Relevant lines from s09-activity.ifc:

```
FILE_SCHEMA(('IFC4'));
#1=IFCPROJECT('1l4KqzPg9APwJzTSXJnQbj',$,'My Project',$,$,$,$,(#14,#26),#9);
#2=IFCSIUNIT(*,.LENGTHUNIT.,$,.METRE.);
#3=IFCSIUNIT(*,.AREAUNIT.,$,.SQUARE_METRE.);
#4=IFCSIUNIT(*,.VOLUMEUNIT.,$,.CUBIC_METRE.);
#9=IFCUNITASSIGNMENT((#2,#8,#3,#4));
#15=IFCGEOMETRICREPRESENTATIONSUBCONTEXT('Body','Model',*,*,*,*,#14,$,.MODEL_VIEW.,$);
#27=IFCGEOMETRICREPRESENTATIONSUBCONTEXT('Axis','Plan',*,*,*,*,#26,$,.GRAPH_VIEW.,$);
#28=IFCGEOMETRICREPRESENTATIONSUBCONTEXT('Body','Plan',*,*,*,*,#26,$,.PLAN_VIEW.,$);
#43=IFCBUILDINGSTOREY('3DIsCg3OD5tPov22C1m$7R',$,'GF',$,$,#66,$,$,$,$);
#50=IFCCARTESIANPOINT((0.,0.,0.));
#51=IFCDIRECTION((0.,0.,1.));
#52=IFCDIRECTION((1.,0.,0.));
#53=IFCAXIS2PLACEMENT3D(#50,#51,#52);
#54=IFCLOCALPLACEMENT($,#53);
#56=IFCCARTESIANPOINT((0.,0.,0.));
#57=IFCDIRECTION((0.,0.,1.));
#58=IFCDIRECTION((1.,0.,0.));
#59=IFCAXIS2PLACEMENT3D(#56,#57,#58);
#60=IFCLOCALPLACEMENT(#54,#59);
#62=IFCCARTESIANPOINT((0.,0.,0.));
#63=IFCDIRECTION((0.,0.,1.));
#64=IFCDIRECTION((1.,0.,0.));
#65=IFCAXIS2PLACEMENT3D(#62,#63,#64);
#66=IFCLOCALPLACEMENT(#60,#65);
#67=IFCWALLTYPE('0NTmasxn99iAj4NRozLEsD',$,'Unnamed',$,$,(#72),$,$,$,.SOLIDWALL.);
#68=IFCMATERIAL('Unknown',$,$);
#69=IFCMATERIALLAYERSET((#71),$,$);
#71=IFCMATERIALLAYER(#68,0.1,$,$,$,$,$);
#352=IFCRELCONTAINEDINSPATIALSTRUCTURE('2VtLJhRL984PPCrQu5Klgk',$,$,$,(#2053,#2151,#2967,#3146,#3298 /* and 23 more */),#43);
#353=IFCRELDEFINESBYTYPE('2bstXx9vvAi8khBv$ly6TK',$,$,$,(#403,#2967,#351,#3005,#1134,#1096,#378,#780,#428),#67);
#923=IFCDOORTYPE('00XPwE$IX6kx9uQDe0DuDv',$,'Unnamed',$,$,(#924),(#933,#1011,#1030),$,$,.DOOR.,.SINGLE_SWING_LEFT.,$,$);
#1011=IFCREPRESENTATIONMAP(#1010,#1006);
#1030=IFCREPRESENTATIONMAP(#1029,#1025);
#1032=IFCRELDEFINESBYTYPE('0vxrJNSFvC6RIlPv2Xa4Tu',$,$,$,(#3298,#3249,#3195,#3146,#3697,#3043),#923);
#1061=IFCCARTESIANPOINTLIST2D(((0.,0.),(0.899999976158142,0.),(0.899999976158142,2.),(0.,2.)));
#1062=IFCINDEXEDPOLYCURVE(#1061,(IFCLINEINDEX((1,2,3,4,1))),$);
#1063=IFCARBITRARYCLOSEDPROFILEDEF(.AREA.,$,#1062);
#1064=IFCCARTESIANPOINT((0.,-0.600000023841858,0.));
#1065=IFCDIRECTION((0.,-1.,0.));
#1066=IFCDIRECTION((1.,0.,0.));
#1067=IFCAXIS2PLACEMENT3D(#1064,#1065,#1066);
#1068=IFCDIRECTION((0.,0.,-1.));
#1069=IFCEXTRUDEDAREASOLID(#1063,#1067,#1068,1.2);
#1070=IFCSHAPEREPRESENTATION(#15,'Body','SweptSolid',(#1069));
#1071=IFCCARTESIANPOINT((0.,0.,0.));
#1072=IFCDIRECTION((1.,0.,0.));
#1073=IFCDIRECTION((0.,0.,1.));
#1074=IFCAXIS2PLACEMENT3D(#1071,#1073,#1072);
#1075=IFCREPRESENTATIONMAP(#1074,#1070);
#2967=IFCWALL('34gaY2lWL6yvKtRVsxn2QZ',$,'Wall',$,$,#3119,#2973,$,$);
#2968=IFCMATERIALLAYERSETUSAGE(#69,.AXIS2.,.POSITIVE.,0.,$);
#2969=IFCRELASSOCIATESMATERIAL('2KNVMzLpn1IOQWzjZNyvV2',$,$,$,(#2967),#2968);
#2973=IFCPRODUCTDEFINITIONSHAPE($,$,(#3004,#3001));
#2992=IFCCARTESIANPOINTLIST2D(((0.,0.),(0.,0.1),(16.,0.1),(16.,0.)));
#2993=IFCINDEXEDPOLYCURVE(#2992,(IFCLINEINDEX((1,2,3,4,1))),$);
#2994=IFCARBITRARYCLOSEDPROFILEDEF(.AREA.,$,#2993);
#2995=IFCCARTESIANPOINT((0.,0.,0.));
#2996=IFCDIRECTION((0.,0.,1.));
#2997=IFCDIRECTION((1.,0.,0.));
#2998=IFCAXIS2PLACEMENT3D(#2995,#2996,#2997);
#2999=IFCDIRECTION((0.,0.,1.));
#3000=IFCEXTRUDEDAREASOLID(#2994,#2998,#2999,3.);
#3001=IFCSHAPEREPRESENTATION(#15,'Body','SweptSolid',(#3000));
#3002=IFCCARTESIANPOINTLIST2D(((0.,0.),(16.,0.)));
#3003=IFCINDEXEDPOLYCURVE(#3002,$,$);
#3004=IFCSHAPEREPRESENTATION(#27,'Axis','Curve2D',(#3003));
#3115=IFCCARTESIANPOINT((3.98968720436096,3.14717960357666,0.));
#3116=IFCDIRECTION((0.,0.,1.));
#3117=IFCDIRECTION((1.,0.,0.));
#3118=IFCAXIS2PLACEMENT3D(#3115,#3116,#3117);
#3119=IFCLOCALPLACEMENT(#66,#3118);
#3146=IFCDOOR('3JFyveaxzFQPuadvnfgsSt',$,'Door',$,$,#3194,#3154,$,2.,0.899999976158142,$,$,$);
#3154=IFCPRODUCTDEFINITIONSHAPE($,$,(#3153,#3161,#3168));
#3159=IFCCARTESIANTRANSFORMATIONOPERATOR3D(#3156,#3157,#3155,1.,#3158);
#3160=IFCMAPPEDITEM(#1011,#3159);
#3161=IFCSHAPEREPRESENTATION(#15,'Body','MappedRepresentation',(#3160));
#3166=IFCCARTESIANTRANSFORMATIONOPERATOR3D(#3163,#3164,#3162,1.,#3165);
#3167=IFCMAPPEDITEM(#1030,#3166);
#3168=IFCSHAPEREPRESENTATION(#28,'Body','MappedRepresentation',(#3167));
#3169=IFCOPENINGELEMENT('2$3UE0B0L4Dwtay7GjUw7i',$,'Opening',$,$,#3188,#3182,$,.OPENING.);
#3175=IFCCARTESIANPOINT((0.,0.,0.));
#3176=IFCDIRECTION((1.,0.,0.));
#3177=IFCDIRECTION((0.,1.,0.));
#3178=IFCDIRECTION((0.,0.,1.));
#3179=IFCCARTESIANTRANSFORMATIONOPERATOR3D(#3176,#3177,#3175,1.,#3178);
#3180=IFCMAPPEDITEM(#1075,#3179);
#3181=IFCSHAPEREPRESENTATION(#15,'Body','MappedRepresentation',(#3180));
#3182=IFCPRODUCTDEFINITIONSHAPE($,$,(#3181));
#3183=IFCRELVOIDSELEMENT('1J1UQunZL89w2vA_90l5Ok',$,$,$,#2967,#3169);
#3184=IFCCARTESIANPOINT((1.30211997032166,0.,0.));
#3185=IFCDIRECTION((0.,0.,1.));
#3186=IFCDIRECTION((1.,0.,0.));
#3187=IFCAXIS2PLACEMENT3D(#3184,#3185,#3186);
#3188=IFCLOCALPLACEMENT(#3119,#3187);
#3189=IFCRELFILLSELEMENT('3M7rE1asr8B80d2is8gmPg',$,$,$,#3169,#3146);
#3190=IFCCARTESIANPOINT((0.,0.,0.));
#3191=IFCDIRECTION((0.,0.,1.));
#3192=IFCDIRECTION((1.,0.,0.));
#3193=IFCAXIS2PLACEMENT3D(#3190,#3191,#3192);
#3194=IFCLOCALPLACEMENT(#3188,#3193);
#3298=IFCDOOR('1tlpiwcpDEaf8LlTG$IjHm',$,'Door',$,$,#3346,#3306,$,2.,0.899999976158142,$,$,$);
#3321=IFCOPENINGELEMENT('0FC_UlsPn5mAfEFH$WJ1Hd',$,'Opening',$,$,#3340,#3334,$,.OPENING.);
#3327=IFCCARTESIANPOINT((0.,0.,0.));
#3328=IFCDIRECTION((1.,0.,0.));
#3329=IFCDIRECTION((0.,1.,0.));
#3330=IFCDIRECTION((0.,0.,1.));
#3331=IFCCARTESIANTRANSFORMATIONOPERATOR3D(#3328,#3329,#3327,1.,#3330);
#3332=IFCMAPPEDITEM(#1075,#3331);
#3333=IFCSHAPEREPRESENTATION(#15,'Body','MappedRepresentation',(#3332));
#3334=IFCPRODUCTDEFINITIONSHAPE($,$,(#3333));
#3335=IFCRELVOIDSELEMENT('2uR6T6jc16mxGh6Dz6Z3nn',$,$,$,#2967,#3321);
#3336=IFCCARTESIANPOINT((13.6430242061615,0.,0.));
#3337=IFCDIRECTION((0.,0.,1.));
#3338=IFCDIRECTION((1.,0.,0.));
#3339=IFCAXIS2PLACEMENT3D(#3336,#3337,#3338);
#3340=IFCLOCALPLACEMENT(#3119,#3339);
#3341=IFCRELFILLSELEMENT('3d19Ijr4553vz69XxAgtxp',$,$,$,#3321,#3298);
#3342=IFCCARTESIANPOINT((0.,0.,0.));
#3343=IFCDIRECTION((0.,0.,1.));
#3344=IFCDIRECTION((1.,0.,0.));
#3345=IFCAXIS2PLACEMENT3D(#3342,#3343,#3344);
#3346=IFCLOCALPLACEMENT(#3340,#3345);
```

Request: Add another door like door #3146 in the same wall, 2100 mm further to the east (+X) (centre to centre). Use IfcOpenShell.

```python
import ifcopenshell
import ifcopenshell.api.feature
import ifcopenshell.api.geometry
import ifcopenshell.api.root
import ifcopenshell.geom
import ifcopenshell.util.element
import ifcopenshell.util.placement
import ifcopenshell.util.shape
import ifcopenshell.util.unit

model = ifcopenshell.open("s09-activity.ifc")
unit_scale = ifcopenshell.util.unit.calculate_unit_scale(model)
settings = ifcopenshell.geom.settings()


def volume(element):
    """Net volume in cubic metres, openings subtracted."""
    shape = ifcopenshell.geom.create_shape(settings, element)
    return ifcopenshell.util.shape.get_volume(shape.geometry)


door = model.by_id(3146)
opening = door.FillsVoids[0].RelatingOpeningElement
wall = opening.VoidsElements[0].RelatingBuildingElement
before = volume(wall)
shift = ifcopenshell.util.placement.get_local_placement(wall.ObjectPlacement)[:3, 0] * 2.1 / unit_scale

# copy_class copies the void relationship, type, container and properties, but no geometry.
new_opening = ifcopenshell.api.root.copy_class(model, product=opening)
new_opening.Representation = ifcopenshell.util.element.copy_deep(
    model, opening.Representation, exclude=["IfcGeometricRepresentationContext", "IfcRepresentationMap"]
)
new_door = ifcopenshell.api.root.copy_class(model, product=door)
new_door.Representation = ifcopenshell.util.element.copy_deep(
    model, door.Representation, exclude=["IfcGeometricRepresentationContext", "IfcRepresentationMap"]
)
ifcopenshell.api.feature.add_filling(model, opening=new_opening, element=new_door)

for old, new in ((opening, new_opening), (door, new_door)):
    matrix = ifcopenshell.util.placement.get_local_placement(old.ObjectPlacement)
    matrix[:3, 3] += shift
    ifcopenshell.api.geometry.edit_object_placement(model, product=new, matrix=matrix, is_si=False)

after = volume(wall)

print(f"wall volume {before:.3f} -> {after:.3f} m3")

model.write("s09-activity_edited.ifc")
```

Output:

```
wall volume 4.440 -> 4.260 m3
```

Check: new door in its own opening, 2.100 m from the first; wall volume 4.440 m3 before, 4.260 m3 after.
